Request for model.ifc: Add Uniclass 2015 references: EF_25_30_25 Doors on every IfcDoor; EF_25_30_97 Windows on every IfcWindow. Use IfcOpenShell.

First a look at what the model holds.

```python
import ifcopenshell

model = ifcopenshell.open("model.ifc")
print(model.schema)
print("classifications:", [c.Name for c in model.by_type("IfcClassification")])
for ifc_class in ("IfcDoor", "IfcRoof", "IfcStair", "IfcWall", "IfcWindow"):
    print(ifc_class, len(model.by_type(ifc_class)))
```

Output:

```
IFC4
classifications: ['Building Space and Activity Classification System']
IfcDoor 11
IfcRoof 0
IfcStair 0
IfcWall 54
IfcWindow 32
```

```python
import ifcopenshell
import ifcopenshell.api.classification

model = ifcopenshell.open("model.ifc")

system = ifcopenshell.api.classification.add_classification(model, classification="Uniclass 2015")

codes = {
    "IfcDoor": ("EF_25_30_25", "Doors"),
    "IfcWindow": ("EF_25_30_97", "Windows"),
}
for ifc_class, (code, name) in codes.items():
    products = model.by_type(ifc_class)
    ifcopenshell.api.classification.add_reference(
        model, products=products, classification=system, identification=code, name=name
    )
    print(code, len(products))

model.write("model_rev.ifc")
```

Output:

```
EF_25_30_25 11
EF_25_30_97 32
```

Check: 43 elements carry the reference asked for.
